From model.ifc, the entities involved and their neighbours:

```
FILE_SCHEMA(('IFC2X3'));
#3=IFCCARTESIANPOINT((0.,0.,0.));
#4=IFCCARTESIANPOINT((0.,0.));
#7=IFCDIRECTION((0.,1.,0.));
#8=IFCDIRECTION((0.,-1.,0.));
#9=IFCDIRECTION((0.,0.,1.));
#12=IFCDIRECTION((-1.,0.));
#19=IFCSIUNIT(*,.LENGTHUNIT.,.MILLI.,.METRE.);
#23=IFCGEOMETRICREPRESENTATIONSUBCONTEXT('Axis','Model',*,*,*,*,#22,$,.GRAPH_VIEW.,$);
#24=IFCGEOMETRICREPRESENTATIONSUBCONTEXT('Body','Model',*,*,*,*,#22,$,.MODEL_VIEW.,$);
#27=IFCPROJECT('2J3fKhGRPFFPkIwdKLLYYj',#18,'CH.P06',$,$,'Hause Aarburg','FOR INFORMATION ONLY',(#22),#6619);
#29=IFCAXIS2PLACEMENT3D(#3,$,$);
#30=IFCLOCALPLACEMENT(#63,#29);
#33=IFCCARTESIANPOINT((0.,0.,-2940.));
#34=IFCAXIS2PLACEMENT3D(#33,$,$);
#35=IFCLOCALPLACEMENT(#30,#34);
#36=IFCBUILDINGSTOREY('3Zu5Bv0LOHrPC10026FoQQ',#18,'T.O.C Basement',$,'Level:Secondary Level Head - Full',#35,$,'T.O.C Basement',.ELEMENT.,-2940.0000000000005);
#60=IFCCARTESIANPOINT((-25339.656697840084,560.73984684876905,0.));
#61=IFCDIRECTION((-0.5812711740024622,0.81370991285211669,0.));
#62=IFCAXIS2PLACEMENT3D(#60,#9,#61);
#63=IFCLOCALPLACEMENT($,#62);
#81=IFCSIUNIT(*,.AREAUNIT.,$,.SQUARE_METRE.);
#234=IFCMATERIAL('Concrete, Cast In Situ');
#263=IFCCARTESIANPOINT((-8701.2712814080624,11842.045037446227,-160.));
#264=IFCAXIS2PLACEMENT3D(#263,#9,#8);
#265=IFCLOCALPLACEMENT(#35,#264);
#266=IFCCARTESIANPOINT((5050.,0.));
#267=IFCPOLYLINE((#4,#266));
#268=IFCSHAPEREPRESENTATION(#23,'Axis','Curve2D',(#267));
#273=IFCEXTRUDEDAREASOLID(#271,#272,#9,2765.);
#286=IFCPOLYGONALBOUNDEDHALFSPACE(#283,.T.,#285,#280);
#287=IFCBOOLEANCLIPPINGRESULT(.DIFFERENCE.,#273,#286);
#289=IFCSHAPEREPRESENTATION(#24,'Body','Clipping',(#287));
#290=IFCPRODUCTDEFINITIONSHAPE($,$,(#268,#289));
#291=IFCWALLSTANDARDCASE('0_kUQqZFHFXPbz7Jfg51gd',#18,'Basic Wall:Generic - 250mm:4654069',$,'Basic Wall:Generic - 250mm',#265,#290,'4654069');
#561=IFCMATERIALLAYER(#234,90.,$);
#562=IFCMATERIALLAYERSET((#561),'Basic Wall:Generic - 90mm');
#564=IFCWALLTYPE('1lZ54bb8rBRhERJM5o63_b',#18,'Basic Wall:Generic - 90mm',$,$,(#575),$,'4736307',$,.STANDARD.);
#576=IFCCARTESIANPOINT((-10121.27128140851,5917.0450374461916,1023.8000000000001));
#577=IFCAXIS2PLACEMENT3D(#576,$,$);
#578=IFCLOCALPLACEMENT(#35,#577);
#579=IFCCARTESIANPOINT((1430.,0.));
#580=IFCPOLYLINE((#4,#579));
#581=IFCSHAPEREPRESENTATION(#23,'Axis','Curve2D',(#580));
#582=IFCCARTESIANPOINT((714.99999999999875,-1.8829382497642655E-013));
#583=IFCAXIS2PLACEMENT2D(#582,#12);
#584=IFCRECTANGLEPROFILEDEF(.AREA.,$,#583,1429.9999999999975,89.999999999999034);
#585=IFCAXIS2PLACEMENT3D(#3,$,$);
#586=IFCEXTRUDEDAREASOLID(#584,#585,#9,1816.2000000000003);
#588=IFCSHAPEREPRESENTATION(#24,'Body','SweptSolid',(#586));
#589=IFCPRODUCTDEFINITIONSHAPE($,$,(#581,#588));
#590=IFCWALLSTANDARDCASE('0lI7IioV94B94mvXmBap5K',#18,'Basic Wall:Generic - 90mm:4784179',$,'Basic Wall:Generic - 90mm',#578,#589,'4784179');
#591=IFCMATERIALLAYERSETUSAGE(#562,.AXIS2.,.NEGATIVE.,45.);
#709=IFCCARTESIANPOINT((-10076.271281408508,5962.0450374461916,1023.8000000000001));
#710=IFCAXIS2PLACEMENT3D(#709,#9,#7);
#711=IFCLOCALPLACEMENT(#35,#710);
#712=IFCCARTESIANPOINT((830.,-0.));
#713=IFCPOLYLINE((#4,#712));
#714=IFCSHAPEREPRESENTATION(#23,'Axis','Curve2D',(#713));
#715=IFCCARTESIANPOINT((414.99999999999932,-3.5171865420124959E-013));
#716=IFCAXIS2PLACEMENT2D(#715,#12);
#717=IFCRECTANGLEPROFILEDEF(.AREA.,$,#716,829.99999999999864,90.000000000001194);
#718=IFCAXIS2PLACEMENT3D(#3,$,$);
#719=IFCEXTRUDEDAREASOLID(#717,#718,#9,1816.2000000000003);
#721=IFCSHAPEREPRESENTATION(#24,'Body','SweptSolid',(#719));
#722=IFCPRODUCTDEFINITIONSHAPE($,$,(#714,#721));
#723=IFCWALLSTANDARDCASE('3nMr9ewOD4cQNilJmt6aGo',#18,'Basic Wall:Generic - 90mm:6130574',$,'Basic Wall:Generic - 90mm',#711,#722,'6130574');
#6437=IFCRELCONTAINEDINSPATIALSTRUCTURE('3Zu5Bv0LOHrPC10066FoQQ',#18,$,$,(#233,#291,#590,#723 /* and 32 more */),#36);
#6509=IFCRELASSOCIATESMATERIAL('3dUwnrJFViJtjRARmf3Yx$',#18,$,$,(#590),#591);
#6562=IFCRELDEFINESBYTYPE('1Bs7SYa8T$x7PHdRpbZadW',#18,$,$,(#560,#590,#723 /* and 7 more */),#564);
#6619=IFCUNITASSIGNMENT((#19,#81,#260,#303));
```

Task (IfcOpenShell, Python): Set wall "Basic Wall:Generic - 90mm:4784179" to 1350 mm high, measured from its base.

```python
import ifcopenshell
import ifcopenshell.geom
import ifcopenshell.util.representation
import ifcopenshell.util.shape
import ifcopenshell.util.unit

model = ifcopenshell.open("model.ifc")
unit_scale = ifcopenshell.util.unit.calculate_unit_scale(model)
settings = ifcopenshell.geom.settings()


def volume(element):
    """Net volume in cubic metres, openings subtracted."""
    shape = ifcopenshell.geom.create_shape(settings, element)
    return ifcopenshell.util.shape.get_volume(shape.geometry)


wall = model.by_guid("0lI7IioV94B94mvXmBap5K")
before = volume(wall)

body = ifcopenshell.util.representation.get_representation(wall, "Model", "Body")
solid = body.Items[0]
old_height = solid.Depth
solid.Depth = 1.35 / unit_scale
after = volume(wall)

print(f"height {old_height:g} -> {solid.Depth:g}, volume {before:.3f} -> {after:.3f} m3")

model.write("model-out.ifc")
```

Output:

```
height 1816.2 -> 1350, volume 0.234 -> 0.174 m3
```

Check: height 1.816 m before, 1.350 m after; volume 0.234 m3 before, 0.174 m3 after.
